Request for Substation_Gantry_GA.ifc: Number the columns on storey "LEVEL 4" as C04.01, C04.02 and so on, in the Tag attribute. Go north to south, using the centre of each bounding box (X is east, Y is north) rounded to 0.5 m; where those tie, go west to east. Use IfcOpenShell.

First a look at what the model holds.

```python
import ifcopenshell
import ifcopenshell.util.element
import ifcopenshell.util.placement

model = ifcopenshell.open("Substation_Gantry_GA.ifc")
print(model.schema)
storey = next(s for s in model.by_type("IfcBuildingStorey") if s.Name == "LEVEL 4")
columns = [e for e in ifcopenshell.util.element.get_decomposition(storey) if e.is_a("IfcColumn")]
for e in sorted(columns, key=lambda e: e.id()):
    origin = ifcopenshell.util.placement.get_local_placement(e.ObjectPlacement)[:3, 3]
    print(e.id(), e.Tag, e.Name, origin.round(2) + 0.0, sep=" | ")
```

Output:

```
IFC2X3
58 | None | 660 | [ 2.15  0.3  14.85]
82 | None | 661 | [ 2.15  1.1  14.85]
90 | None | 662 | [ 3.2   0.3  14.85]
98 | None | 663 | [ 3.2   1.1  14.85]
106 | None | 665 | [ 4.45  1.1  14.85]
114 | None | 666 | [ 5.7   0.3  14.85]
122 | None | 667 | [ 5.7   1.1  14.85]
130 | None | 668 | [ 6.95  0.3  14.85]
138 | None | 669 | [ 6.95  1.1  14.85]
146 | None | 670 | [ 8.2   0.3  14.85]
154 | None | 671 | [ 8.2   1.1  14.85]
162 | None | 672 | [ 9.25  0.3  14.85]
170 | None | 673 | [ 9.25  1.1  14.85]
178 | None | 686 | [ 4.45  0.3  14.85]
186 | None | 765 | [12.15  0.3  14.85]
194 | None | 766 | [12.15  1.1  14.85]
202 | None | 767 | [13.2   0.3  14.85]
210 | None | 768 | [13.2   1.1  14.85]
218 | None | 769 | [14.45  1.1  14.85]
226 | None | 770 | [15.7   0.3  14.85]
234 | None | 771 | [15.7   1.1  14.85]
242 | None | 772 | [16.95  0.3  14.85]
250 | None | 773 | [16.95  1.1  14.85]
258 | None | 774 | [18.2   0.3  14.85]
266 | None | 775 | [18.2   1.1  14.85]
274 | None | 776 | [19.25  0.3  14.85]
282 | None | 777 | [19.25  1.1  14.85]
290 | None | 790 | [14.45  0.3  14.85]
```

```python
import ifcopenshell
import ifcopenshell.geom
import ifcopenshell.util.element
import ifcopenshell.util.shape

model = ifcopenshell.open("Substation_Gantry_GA.ifc")
settings = ifcopenshell.geom.settings()
settings.set("use-world-coords", True)


def centre(element):
    shape = ifcopenshell.geom.create_shape(settings, element)
    return ifcopenshell.util.shape.get_bbox_centroid(shape.geometry)


storey = next(s for s in model.by_type("IfcBuildingStorey") if s.Name == "LEVEL 4")
columns = [e for e in ifcopenshell.util.element.get_decomposition(storey) if e.is_a("IfcColumn")]

# Insertion points can sit at a corner or the storey origin, so sort by the geometry (in metres).
centres = {e: centre(e) for e in columns}
columns.sort(key=lambda e: (-round(centres[e][1] / 0.5), centres[e][0]))

for i, e in enumerate(columns, start=1):
    number = f"C04.{i:02d}"
    e.Tag = number
    print(e.id(), number)

model.write("Substation_Gantry_GA_v2.ifc")
```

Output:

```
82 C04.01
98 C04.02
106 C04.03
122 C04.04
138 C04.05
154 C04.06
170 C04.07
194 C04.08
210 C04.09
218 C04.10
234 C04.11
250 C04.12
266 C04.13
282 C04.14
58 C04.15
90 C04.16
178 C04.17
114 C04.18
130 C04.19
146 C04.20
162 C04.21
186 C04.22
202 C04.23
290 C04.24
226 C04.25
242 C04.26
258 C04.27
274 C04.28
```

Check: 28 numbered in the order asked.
